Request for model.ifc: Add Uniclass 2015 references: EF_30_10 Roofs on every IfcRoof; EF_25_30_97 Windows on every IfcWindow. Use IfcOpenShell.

First a look at what the model holds.

```python
import ifcopenshell

model = ifcopenshell.open("model.ifc")
print(model.schema)
print("classifications:", [c.Name for c in model.by_type("IfcClassification")])
for ifc_class in ("IfcDoor", "IfcRoof", "IfcStair", "IfcWall", "IfcWindow"):
    print(ifc_class, len(model.by_type(ifc_class)))
```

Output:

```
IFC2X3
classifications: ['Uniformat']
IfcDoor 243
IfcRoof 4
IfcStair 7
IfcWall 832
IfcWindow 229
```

```python
import ifcopenshell
import ifcopenshell.api.classification

model = ifcopenshell.open("model.ifc")

# IFC2X3 requires Source and Edition and has no link from the project to the system.
system = model.create_entity("IfcClassification", Source="NBS", Edition="2015", Name="Uniclass 2015")

codes = {
    "IfcRoof": ("EF_30_10", "Roofs"),
    "IfcWindow": ("EF_25_30_97", "Windows"),
}
for ifc_class, (code, name) in codes.items():
    products = model.by_type(ifc_class)
    ifcopenshell.api.classification.add_reference(
        model, products=products, classification=system, identification=code, name=name
    )
    print(code, len(products))

model.write("model_edited.ifc")
```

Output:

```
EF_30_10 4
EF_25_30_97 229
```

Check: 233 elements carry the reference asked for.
